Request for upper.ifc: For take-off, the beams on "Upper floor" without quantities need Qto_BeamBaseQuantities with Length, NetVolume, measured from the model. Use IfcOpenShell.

First a look at what the model holds.

```python
import ifcopenshell
import ifcopenshell.util.element
import ifcopenshell.util.unit

model = ifcopenshell.open("upper.ifc")
print(model.schema)
for unit_type in ("LENGTHUNIT", "AREAUNIT", "VOLUMEUNIT"):
    print(unit_type, ifcopenshell.util.unit.calculate_unit_scale(model, unit_type))
storey = next(s for s in model.by_type("IfcBuildingStorey") if s.Name == "Upper floor")
beams = [e for e in ifcopenshell.util.element.get_decomposition(storey) if e.is_a("IfcBeam")]
for e in sorted(beams, key=lambda e: e.id()):
    print(e.id(), e.is_a(), e.Name, list(ifcopenshell.util.element.get_psets(e, qtos_only=True)), sep=" | ")
```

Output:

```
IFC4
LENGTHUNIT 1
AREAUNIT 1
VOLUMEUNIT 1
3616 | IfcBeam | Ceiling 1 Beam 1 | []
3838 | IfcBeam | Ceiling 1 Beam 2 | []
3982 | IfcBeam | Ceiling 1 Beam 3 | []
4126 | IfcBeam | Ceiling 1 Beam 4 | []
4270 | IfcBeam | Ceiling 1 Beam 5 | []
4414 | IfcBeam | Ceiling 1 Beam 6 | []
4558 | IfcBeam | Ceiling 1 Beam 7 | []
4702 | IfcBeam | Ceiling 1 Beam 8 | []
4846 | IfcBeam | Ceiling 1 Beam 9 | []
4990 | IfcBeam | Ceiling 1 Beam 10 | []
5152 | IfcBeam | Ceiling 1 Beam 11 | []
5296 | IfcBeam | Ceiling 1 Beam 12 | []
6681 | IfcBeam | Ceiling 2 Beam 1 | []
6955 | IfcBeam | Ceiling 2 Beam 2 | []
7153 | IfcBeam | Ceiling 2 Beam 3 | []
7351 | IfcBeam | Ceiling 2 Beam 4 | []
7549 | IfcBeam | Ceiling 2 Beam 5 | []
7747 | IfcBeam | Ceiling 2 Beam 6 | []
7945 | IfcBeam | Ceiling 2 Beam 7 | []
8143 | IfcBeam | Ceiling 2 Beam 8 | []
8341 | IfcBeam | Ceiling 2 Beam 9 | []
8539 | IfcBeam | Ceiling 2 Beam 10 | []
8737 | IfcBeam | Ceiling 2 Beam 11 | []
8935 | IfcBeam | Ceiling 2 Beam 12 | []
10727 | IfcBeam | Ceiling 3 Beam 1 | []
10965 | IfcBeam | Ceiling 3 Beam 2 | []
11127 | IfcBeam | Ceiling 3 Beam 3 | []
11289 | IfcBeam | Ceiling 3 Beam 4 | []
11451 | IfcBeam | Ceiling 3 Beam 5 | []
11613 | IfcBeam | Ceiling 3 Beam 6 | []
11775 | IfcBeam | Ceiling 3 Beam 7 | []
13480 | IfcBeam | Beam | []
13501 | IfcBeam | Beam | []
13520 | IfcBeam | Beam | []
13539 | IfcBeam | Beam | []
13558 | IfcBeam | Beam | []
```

```python
import ifcopenshell
import ifcopenshell.api.pset
import ifcopenshell.geom
import ifcopenshell.util.element
import ifcopenshell.util.shape
import ifcopenshell.util.unit

model = ifcopenshell.open("upper.ifc")
unit_scale = ifcopenshell.util.unit.calculate_unit_scale(model)
volume_scale = ifcopenshell.util.unit.calculate_unit_scale(model, "VOLUMEUNIT")
settings = ifcopenshell.geom.settings()

storey = next(s for s in model.by_type("IfcBuildingStorey") if s.Name == "Upper floor")
beams = [e for e in ifcopenshell.util.element.get_decomposition(storey) if e.is_a("IfcBeam")]

for e in sorted(beams, key=lambda e: e.id()):
    if ifcopenshell.util.element.get_psets(e, qtos_only=True, should_inherit=False):
        continue
    # Geometry comes back in metres, in the element's own axes.
    shape = ifcopenshell.geom.create_shape(settings, e)
    values = {
        "Length": ifcopenshell.util.shape.get_max_xyz(shape.geometry) / unit_scale,
        "NetVolume": ifcopenshell.util.shape.get_volume(shape.geometry) / volume_scale,
    }
    qto = ifcopenshell.api.pset.add_qto(model, product=e, name="Qto_BeamBaseQuantities")
    ifcopenshell.api.pset.edit_qto(model, qto=qto, properties=values)
    print(e.id(), {k: round(v, 3) for k, v in values.items()})

model.write("upper-out.ifc")
```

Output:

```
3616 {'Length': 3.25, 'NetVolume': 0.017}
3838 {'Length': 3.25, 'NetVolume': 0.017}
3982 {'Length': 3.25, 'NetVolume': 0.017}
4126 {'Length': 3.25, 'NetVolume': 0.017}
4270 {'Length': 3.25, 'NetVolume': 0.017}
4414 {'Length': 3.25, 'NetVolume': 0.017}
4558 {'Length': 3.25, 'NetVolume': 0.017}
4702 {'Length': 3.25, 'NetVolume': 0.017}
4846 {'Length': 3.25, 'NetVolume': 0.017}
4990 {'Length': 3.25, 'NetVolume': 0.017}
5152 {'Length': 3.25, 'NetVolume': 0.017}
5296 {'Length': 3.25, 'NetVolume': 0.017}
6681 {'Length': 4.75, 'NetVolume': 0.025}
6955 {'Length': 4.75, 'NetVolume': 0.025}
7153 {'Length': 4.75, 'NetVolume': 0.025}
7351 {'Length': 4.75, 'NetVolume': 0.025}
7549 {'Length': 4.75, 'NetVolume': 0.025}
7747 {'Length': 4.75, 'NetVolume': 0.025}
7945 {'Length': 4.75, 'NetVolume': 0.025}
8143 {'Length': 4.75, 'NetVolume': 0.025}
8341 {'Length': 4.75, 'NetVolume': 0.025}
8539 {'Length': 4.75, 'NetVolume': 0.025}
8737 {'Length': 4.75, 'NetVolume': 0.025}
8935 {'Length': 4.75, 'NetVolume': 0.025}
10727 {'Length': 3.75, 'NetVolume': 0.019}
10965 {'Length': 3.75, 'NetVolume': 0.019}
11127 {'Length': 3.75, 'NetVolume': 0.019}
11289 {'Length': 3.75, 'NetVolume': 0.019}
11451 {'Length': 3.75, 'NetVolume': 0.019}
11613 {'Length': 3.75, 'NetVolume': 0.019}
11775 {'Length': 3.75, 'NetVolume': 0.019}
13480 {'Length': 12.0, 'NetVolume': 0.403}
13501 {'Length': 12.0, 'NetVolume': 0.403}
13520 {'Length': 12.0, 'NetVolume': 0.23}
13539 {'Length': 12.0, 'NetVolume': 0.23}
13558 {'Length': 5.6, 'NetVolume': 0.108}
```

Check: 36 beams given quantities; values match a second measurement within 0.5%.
